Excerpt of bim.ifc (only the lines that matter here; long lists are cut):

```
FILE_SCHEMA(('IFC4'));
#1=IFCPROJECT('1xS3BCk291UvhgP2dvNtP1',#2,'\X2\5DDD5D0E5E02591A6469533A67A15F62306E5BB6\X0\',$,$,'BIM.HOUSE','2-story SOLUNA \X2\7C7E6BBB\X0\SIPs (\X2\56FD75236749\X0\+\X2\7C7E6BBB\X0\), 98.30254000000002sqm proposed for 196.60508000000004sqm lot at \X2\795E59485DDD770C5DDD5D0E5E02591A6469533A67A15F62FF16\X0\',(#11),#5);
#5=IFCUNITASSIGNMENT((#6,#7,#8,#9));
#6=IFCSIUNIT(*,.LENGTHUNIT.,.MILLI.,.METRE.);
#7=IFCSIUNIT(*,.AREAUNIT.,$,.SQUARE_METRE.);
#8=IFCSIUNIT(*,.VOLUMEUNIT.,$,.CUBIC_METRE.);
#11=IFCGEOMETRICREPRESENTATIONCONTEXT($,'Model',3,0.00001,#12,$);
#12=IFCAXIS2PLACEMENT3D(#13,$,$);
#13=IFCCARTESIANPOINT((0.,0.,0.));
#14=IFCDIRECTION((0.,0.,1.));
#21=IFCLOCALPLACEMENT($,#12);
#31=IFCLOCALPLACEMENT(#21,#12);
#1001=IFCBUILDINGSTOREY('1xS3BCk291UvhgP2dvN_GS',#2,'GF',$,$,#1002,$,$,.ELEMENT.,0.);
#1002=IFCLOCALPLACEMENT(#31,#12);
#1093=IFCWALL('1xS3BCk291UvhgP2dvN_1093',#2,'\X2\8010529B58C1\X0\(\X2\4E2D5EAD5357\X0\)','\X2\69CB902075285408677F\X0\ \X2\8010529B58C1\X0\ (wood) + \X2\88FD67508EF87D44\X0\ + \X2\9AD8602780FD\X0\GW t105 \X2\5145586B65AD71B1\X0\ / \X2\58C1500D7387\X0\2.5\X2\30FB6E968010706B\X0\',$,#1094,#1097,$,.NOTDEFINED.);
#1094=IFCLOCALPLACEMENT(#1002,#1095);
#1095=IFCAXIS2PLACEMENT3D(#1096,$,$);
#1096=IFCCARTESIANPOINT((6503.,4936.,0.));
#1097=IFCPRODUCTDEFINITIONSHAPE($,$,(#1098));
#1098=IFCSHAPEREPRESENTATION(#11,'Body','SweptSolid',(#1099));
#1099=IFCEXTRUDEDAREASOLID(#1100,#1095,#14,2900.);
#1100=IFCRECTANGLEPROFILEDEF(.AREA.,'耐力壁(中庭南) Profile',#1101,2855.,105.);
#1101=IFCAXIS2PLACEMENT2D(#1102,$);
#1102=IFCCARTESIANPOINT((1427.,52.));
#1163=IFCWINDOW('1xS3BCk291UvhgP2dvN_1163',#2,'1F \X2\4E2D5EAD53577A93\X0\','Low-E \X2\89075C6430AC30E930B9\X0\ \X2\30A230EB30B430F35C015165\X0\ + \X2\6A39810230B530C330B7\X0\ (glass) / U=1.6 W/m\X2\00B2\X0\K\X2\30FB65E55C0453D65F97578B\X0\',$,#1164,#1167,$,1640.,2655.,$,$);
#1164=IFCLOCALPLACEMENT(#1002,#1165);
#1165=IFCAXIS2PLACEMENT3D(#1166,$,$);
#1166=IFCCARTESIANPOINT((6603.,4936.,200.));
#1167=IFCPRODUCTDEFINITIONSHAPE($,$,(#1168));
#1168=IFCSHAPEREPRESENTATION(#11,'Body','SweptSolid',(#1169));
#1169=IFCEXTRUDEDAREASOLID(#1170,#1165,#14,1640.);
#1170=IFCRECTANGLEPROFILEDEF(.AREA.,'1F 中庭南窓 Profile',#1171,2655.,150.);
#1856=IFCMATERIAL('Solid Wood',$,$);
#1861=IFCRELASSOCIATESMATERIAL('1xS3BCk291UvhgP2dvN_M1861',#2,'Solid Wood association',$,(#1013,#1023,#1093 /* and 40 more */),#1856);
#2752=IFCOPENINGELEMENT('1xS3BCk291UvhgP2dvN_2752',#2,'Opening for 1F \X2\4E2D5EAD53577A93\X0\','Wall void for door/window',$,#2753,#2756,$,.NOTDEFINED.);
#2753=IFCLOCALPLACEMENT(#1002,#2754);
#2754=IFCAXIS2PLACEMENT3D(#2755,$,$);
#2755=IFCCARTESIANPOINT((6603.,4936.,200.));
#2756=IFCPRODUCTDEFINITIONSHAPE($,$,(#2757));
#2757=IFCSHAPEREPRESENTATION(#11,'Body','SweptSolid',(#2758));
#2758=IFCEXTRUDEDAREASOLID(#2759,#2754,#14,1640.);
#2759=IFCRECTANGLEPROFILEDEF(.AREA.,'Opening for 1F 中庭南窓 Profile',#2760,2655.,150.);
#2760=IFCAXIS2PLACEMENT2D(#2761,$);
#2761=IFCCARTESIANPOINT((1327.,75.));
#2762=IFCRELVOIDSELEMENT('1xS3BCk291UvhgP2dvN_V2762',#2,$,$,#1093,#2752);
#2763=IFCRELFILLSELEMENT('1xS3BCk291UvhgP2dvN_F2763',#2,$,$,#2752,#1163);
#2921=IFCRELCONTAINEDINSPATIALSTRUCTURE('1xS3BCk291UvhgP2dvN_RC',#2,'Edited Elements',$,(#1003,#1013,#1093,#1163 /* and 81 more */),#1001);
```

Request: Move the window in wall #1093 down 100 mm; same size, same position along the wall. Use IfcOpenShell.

```python
import numpy as np
import ifcopenshell
import ifcopenshell.api.geometry
import ifcopenshell.util.placement
import ifcopenshell.util.unit

model = ifcopenshell.open("bim.ifc")
unit_scale = ifcopenshell.util.unit.calculate_unit_scale(model)

window = model.by_guid("1xS3BCk291UvhgP2dvN_1163")
opening = window.FillsVoids[0].RelatingOpeningElement
dz = -0.1 / unit_scale

shift = np.array([0.0, 0.0, dz])
# The window is not placed relative to its opening, so move both.
for product in (opening, window):
    matrix = ifcopenshell.util.placement.get_local_placement(product.ObjectPlacement)
    matrix[:3, 3] += shift
    ifcopenshell.api.geometry.edit_object_placement(model, product=product, matrix=matrix, is_si=False)

print(f"moved by {dz * unit_scale:+.3f} m")

model.write("bim_rev.ifc")
```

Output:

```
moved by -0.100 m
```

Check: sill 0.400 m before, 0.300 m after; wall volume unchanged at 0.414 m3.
